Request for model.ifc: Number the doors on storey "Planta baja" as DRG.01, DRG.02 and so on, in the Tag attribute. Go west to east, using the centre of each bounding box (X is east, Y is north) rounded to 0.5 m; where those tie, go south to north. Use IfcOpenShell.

First a look at what the model holds.

```python
import ifcopenshell
import ifcopenshell.util.element
import ifcopenshell.util.placement

model = ifcopenshell.open("model.ifc")
print(model.schema)
storey = next(s for s in model.by_type("IfcBuildingStorey") if s.Name == "Planta baja")
doors = [e for e in ifcopenshell.util.element.get_decomposition(storey) if e.is_a("IfcDoor")]
for e in sorted(doors, key=lambda e: e.id()):
    origin = ifcopenshell.util.placement.get_local_placement(e.ObjectPlacement)[:3, 3]
    print(e.id(), e.Tag, e.Name, origin.round(2) + 0.0, sep=" | ")
```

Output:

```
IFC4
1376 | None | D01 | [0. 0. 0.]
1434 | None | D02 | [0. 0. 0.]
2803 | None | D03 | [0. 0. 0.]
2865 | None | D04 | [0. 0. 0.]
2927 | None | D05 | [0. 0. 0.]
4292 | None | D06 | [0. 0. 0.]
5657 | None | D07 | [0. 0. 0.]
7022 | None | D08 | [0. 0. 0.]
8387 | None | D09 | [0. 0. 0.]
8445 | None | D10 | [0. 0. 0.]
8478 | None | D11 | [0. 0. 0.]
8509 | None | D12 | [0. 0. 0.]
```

```python
import ifcopenshell
import ifcopenshell.geom
import ifcopenshell.util.element
import ifcopenshell.util.shape

model = ifcopenshell.open("model.ifc")
settings = ifcopenshell.geom.settings()
settings.set("use-world-coords", True)


def centre(element):
    shape = ifcopenshell.geom.create_shape(settings, element)
    return ifcopenshell.util.shape.get_bbox_centroid(shape.geometry)


storey = next(s for s in model.by_type("IfcBuildingStorey") if s.Name == "Planta baja")
doors = [e for e in ifcopenshell.util.element.get_decomposition(storey) if e.is_a("IfcDoor")]

# Insertion points can sit at a corner or the storey origin, so sort by the geometry (in metres).
centres = {e: centre(e) for e in doors}
doors.sort(key=lambda e: (round(centres[e][0] / 0.5), centres[e][1]))

for i, e in enumerate(doors, start=1):
    number = f"DRG.{i:02d}"
    e.Tag = number
    print(e.id(), number)

model.write("model-out.ifc")
```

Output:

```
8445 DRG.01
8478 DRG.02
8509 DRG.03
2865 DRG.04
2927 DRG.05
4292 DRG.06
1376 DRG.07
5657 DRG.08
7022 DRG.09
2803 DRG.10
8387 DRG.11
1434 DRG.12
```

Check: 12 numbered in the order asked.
